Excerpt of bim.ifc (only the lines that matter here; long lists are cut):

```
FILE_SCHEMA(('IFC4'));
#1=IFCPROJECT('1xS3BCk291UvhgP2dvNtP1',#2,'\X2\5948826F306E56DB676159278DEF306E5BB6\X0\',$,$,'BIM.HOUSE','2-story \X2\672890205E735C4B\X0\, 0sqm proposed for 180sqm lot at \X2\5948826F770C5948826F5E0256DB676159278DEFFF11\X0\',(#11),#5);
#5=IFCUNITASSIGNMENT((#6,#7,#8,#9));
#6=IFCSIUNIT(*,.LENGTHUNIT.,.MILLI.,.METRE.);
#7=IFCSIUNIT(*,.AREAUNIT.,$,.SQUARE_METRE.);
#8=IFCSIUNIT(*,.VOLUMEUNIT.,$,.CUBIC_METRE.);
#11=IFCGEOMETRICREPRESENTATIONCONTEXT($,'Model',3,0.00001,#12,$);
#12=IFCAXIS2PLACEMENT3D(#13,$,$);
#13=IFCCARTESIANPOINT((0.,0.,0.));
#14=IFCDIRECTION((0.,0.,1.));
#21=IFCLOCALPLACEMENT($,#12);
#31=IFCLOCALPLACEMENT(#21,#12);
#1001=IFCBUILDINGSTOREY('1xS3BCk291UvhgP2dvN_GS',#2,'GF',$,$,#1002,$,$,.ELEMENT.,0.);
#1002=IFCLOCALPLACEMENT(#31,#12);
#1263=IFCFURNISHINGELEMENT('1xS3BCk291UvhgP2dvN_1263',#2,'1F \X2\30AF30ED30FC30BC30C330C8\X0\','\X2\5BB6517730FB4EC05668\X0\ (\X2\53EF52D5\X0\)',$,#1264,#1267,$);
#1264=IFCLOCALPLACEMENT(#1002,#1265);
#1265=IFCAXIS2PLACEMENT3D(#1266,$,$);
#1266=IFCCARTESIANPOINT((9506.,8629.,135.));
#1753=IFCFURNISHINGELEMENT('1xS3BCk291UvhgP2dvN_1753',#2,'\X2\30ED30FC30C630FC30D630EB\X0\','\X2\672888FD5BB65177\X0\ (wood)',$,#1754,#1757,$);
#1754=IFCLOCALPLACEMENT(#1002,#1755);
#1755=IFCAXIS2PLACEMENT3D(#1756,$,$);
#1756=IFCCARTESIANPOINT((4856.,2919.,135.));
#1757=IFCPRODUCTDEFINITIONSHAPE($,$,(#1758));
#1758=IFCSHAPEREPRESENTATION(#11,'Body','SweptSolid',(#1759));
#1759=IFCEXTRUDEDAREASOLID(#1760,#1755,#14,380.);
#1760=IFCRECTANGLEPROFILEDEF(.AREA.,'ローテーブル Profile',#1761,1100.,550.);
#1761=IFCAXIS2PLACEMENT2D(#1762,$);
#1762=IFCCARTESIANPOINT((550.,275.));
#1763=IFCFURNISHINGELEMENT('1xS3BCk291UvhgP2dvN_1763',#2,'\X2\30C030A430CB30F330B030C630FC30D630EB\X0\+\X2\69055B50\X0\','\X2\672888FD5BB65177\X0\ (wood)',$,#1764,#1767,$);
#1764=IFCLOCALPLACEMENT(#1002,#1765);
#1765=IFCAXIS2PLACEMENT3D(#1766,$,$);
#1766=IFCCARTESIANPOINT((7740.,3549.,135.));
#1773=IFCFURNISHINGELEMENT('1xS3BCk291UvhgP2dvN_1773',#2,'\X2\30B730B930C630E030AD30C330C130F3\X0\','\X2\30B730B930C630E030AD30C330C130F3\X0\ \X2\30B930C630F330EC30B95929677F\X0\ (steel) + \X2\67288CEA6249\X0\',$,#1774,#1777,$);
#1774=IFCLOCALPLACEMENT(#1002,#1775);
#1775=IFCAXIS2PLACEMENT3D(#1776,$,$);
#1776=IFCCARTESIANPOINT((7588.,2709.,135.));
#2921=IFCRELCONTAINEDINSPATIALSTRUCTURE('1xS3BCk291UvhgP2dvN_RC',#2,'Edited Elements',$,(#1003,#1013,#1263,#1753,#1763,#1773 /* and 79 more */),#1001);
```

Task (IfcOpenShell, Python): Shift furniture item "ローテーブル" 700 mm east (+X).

```python
import ifcopenshell
import ifcopenshell.api.geometry
import ifcopenshell.util.placement

model = ifcopenshell.open("bim.ifc")

item = model.by_guid("1xS3BCk291UvhgP2dvN_1753")
matrix = ifcopenshell.util.placement.get_local_placement(item.ObjectPlacement)
matrix[0, 3] += 700.0
ifcopenshell.api.geometry.edit_object_placement(model, product=item, matrix=matrix, is_si=False)

print(ifcopenshell.util.placement.get_local_placement(item.ObjectPlacement).round(3) + 0.0)

model.write("bim_v2.ifc")
```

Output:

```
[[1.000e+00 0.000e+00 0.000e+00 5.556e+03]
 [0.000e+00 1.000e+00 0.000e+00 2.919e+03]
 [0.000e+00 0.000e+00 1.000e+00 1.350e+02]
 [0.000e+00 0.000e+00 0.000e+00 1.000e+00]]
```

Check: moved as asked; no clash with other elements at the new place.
